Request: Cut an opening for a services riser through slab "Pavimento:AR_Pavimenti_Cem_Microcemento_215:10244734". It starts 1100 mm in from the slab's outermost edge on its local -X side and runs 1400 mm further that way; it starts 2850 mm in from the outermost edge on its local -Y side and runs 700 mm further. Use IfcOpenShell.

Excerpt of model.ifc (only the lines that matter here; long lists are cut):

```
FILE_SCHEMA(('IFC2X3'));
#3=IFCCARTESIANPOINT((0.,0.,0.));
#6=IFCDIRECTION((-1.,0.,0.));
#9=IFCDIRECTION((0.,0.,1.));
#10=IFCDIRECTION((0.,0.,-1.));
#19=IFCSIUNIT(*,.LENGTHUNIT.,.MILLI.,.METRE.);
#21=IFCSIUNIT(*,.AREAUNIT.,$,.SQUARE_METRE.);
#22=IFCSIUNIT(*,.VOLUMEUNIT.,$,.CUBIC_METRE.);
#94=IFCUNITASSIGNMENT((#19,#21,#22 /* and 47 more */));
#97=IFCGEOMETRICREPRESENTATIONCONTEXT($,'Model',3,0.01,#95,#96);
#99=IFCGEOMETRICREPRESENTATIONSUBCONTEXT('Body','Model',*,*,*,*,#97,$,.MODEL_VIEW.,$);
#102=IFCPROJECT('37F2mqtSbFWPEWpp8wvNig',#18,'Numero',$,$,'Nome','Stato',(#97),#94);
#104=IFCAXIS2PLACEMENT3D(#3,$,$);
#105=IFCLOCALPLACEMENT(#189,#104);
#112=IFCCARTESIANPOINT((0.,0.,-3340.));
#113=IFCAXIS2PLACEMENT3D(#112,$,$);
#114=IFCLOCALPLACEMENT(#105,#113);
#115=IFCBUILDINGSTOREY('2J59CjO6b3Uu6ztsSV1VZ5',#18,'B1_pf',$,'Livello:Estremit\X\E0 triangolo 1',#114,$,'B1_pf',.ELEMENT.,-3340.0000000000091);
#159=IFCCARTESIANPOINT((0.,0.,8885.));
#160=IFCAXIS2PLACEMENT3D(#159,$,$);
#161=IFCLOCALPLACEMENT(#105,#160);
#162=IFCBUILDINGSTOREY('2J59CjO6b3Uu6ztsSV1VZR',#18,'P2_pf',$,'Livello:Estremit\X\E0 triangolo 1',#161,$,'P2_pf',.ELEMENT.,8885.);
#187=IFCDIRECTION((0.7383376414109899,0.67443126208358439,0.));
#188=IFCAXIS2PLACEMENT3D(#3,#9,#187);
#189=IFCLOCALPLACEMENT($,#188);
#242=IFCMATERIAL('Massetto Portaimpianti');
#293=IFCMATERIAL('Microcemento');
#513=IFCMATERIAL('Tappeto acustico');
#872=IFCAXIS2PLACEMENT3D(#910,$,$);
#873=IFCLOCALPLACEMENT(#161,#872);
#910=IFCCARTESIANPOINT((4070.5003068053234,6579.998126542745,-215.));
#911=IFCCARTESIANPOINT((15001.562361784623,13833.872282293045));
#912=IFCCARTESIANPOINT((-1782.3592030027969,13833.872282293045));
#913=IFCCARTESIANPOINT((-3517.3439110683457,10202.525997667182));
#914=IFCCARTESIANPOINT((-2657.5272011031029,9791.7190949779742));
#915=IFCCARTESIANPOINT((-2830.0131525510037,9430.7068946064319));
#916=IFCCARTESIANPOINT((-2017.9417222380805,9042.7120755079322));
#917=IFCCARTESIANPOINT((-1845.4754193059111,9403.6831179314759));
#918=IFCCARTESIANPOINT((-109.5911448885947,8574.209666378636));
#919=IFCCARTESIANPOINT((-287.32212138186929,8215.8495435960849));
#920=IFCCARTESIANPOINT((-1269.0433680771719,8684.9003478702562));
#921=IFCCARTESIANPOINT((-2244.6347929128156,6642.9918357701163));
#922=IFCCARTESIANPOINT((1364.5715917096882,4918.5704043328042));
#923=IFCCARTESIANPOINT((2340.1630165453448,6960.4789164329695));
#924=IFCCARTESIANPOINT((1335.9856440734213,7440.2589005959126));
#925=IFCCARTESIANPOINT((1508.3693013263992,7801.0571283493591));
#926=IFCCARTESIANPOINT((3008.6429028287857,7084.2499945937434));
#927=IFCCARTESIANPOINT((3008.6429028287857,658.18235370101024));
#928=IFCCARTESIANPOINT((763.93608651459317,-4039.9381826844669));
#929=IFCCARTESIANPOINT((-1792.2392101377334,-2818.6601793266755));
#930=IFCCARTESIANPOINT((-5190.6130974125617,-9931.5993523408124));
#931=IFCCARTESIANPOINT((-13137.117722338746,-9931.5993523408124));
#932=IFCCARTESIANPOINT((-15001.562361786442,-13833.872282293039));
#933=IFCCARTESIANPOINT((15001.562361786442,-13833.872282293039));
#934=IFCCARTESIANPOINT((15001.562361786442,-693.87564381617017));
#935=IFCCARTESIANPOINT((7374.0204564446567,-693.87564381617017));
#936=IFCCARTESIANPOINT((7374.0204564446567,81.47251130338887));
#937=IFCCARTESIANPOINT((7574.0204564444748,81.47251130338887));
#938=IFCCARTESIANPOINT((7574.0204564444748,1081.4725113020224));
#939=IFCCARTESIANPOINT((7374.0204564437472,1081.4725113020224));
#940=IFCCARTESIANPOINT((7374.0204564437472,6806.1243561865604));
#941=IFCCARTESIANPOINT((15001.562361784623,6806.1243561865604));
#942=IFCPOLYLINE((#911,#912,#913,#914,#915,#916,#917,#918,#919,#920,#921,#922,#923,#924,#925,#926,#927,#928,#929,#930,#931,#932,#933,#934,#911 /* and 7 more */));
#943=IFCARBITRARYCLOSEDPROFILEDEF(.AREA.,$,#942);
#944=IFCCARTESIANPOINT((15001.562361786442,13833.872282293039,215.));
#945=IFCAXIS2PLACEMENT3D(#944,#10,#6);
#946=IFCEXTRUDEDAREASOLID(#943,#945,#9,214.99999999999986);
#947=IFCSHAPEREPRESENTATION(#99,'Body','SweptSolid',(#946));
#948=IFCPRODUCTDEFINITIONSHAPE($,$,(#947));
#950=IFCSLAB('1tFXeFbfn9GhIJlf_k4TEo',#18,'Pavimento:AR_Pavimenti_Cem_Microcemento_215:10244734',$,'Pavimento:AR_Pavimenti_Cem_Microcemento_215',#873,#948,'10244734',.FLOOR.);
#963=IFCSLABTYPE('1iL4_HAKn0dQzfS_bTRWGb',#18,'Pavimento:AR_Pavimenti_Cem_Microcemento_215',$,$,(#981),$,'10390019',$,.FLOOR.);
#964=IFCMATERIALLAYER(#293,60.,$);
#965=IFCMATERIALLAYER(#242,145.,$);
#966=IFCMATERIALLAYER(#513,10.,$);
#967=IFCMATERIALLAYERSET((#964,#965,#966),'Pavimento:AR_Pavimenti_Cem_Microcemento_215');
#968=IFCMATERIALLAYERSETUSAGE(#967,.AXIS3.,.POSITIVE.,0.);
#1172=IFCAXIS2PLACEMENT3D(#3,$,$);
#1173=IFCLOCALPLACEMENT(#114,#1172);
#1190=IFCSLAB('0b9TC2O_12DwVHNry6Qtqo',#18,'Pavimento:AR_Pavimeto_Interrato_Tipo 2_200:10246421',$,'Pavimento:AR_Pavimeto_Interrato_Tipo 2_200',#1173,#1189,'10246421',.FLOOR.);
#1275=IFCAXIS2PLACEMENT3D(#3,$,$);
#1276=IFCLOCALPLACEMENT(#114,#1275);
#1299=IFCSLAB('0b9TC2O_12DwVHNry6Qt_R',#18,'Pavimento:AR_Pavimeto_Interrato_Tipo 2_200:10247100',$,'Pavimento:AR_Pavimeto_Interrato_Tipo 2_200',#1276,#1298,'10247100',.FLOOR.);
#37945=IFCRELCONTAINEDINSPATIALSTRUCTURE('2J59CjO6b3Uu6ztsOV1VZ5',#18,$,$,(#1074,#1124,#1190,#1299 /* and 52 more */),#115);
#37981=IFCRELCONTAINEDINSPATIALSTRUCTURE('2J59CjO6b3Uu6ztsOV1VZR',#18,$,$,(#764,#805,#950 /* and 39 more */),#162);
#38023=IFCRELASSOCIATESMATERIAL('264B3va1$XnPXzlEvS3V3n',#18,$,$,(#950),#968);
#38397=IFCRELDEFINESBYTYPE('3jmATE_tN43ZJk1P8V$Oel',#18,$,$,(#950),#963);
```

```python
import numpy as np
import ifcopenshell
import ifcopenshell.api.feature
import ifcopenshell.api.geometry
import ifcopenshell.api.root
import ifcopenshell.geom
import ifcopenshell.util.placement
import ifcopenshell.util.representation
import ifcopenshell.util.shape
import ifcopenshell.util.unit

model = ifcopenshell.open("model.ifc")
unit_scale = ifcopenshell.util.unit.calculate_unit_scale(model)
settings = ifcopenshell.geom.settings()


def volume(element):
    """Net volume in cubic metres, openings subtracted."""
    shape = ifcopenshell.geom.create_shape(settings, element)
    return ifcopenshell.util.shape.get_volume(shape.geometry)


slab = model.by_guid("1tFXeFbfn9GhIJlf_k4TEo")
before = volume(slab)

# Extent in the slab's own axes, in metres. The edges named are its -X and -Y sides.
slab_shape = ifcopenshell.geom.create_shape(settings, slab)
vertices = ifcopenshell.util.shape.get_vertices(slab_shape.geometry)
x_min, y_min, bottom = vertices.min(axis=0)
top = vertices[:, 2].max()

opening = ifcopenshell.api.root.create_entity(model, ifc_class="IfcOpeningElement", name="Services riser opening")
context = ifcopenshell.util.representation.get_context(model, "Model", "Body", "MODEL_VIEW")
width, depth = 1.4, 0.7
outline = [(0.0, 0.0), (width, 0.0), (width, depth), (0.0, depth), (0.0, 0.0)]
# Overshoot both faces by 50 mm so the cut is clean.
shape = ifcopenshell.api.geometry.add_slab_representation(
    model, context=context, depth=top - bottom + 0.1, polyline=outline
)
ifcopenshell.api.geometry.assign_representation(model, product=opening, representation=shape)

matrix = ifcopenshell.util.placement.get_local_placement(slab.ObjectPlacement)
matrix[:, 3] = matrix @ np.append(np.array([x_min + 1.1, y_min + 2.85, bottom - 0.05]) / unit_scale, 1.0)
ifcopenshell.api.geometry.edit_object_placement(model, product=opening, matrix=matrix, is_si=False)
ifcopenshell.api.feature.add_feature(model, feature=opening, element=slab)

after = volume(slab)

print(f"slab volume {before:.3f} -> {after:.3f} m3")

model.write("model_v2.ifc")
```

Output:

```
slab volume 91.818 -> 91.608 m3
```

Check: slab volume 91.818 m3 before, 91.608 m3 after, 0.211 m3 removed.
